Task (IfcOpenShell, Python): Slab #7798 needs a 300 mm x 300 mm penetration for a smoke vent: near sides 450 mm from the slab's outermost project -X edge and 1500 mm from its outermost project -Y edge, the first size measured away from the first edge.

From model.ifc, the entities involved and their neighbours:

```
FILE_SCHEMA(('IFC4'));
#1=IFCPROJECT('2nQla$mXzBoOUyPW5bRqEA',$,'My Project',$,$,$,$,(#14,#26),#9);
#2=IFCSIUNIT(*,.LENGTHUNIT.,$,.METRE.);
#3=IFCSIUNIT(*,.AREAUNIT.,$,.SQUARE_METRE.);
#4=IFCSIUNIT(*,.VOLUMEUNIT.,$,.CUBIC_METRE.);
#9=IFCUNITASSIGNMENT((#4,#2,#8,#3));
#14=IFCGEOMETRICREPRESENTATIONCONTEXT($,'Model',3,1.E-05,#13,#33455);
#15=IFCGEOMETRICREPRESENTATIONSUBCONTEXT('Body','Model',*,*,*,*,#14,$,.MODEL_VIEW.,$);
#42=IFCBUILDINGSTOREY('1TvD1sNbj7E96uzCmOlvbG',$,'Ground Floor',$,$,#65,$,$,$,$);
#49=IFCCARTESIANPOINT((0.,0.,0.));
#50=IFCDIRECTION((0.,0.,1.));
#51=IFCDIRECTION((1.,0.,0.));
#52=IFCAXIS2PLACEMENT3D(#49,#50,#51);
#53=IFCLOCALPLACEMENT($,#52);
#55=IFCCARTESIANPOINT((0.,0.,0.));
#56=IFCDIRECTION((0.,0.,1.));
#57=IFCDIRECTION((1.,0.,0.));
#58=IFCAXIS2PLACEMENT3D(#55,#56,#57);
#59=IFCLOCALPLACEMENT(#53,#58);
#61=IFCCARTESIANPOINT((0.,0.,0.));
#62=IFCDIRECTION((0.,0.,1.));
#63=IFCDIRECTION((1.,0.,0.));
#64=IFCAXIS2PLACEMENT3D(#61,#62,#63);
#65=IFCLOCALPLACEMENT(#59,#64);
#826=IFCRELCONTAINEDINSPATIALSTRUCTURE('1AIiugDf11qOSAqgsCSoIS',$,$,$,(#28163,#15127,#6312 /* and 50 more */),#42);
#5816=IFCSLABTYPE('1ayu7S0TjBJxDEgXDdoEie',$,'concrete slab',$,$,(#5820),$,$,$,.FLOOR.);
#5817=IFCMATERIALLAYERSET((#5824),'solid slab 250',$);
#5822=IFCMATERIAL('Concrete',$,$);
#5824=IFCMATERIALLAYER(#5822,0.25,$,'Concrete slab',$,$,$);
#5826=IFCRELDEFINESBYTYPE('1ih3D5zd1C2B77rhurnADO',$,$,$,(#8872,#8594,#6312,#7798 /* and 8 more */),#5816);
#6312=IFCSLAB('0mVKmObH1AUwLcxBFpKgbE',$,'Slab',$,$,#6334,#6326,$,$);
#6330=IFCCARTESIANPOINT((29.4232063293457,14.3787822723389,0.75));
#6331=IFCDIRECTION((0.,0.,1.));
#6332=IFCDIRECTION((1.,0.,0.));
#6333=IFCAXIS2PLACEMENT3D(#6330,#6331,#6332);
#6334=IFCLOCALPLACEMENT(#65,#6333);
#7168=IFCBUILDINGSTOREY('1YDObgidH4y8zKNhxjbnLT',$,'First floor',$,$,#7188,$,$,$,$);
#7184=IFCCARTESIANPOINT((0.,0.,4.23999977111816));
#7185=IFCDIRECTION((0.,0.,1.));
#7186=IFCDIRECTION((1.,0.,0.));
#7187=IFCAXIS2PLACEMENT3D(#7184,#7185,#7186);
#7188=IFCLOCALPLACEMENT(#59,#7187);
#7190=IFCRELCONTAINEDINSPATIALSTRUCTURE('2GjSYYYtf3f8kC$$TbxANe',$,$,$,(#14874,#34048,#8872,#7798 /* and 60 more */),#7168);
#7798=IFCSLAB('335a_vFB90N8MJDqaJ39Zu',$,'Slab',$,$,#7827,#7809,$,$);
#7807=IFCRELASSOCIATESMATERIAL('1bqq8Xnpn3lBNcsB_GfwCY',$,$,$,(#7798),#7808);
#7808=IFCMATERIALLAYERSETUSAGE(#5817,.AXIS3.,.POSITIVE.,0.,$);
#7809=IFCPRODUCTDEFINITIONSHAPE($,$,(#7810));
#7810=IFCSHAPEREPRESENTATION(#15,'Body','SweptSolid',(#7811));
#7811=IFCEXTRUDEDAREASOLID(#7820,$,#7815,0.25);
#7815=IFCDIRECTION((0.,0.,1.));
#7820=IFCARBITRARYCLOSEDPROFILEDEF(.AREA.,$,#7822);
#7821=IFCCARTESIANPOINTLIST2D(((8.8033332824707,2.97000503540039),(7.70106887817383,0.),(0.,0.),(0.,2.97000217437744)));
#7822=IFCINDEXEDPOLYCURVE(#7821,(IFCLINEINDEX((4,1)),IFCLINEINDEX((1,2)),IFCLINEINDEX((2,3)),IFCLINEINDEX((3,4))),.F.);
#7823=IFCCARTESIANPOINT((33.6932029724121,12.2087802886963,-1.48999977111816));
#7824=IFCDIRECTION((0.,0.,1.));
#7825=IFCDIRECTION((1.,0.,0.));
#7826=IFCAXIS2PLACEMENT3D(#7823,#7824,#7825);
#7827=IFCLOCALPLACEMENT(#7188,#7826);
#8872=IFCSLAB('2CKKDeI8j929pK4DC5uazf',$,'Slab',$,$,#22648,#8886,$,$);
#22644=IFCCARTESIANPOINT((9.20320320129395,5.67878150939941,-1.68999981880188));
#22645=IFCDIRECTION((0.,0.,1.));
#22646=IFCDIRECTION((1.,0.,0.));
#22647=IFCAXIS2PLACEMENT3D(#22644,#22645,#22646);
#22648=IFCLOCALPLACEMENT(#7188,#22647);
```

```python
import numpy as np
import ifcopenshell
import ifcopenshell.api.feature
import ifcopenshell.api.geometry
import ifcopenshell.api.root
import ifcopenshell.geom
import ifcopenshell.util.placement
import ifcopenshell.util.representation
import ifcopenshell.util.shape
import ifcopenshell.util.unit

model = ifcopenshell.open("model.ifc")
unit_scale = ifcopenshell.util.unit.calculate_unit_scale(model)
settings = ifcopenshell.geom.settings()


def volume(element):
    """Net volume in cubic metres, openings subtracted."""
    shape = ifcopenshell.geom.create_shape(settings, element)
    return ifcopenshell.util.shape.get_volume(shape.geometry)


slab = model.by_guid("335a_vFB90N8MJDqaJ39Zu")
before = volume(slab)

# Extent in the slab's own axes, in metres. The edges named are its -X and -Y sides.
slab_shape = ifcopenshell.geom.create_shape(settings, slab)
vertices = ifcopenshell.util.shape.get_vertices(slab_shape.geometry)
x_min, y_min, bottom = vertices.min(axis=0)
top = vertices[:, 2].max()

opening = ifcopenshell.api.root.create_entity(model, ifc_class="IfcOpeningElement", name="Smoke vent opening", predefined_type="OPENING")
context = ifcopenshell.util.representation.get_context(model, "Model", "Body", "MODEL_VIEW")
width, depth = 0.3, 0.3
outline = [(0.0, 0.0), (width, 0.0), (width, depth), (0.0, depth), (0.0, 0.0)]
# Overshoot both faces by 50 mm so the cut is clean.
shape = ifcopenshell.api.geometry.add_slab_representation(
    model, context=context, depth=top - bottom + 0.1, polyline=outline
)
ifcopenshell.api.geometry.assign_representation(model, product=opening, representation=shape)

matrix = ifcopenshell.util.placement.get_local_placement(slab.ObjectPlacement)
matrix[:, 3] = matrix @ np.append(np.array([x_min + 0.45, y_min + 1.5, bottom - 0.05]) / unit_scale, 1.0)
ifcopenshell.api.geometry.edit_object_placement(model, product=opening, matrix=matrix, is_si=False)
ifcopenshell.api.feature.add_feature(model, feature=opening, element=slab)

after = volume(slab)

print(f"slab volume {before:.3f} -> {after:.3f} m3")

model.write("model_updated.ifc")
```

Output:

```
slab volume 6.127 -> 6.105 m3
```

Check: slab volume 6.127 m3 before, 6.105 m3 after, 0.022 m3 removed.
